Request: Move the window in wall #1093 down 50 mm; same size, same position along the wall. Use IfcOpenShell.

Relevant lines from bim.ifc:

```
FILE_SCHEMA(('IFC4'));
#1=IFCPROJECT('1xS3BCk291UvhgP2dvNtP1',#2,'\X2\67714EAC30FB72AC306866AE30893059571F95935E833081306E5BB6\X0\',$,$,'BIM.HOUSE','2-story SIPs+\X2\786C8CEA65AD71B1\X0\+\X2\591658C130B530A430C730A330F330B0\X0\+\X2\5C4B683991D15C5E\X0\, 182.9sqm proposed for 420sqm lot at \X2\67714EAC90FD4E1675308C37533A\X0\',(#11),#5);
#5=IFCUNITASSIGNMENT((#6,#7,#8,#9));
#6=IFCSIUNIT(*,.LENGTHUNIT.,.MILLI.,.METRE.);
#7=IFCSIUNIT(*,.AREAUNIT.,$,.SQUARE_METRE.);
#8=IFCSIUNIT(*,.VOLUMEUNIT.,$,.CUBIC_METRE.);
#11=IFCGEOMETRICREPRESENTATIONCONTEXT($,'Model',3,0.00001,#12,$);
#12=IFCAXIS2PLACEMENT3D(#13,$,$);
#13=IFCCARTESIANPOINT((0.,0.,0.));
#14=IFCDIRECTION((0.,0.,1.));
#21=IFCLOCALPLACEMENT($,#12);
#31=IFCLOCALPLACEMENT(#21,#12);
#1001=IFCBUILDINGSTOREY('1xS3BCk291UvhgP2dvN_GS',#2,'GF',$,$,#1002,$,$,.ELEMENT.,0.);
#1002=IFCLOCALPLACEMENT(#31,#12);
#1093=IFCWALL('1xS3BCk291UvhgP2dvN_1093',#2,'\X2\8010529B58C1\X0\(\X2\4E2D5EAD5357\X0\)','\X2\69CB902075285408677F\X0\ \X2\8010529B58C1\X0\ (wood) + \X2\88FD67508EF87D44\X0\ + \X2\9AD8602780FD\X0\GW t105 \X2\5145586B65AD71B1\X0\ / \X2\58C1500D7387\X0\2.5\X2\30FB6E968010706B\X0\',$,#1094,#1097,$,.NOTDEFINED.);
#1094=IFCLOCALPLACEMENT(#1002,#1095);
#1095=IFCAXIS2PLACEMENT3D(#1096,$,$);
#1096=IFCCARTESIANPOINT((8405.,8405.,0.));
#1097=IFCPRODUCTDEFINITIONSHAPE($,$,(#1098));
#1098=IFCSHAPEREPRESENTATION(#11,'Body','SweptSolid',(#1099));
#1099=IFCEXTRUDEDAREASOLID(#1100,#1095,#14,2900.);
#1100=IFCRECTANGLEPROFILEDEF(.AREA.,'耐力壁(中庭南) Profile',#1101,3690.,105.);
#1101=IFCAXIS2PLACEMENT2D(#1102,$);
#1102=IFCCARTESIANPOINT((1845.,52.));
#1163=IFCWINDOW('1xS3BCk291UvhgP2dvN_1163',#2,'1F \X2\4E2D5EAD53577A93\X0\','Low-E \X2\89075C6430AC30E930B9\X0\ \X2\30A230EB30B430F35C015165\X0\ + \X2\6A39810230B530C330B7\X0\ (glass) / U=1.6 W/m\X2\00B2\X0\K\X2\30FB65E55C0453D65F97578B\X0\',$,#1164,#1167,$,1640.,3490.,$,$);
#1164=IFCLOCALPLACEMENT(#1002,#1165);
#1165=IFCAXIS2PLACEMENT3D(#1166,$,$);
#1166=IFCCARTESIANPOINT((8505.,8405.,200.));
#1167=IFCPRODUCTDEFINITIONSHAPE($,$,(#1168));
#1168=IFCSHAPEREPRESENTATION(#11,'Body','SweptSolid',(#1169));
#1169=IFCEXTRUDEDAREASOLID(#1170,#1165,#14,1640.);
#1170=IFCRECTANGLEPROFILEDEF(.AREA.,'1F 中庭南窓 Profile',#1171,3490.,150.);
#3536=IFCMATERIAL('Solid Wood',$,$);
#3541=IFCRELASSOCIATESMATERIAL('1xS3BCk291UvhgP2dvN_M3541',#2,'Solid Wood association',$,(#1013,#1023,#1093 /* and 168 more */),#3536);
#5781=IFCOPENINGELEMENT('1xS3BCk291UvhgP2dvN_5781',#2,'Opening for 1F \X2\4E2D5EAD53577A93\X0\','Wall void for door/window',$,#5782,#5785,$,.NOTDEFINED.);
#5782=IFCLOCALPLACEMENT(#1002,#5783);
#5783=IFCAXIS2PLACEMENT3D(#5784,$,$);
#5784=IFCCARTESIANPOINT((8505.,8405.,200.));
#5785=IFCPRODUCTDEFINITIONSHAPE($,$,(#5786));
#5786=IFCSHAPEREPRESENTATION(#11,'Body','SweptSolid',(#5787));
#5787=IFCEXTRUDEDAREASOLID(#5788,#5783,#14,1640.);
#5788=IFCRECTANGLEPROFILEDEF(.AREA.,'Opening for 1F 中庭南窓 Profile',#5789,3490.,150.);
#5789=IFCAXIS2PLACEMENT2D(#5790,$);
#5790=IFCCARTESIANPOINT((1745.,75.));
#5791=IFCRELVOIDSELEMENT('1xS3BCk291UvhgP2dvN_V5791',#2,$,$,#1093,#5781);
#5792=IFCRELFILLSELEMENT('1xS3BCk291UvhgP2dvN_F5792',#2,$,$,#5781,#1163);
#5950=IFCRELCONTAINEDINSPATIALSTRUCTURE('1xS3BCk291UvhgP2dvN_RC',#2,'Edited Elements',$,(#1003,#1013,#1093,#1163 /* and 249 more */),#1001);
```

```python
import numpy as np
import ifcopenshell
import ifcopenshell.api.geometry
import ifcopenshell.util.placement
import ifcopenshell.util.unit

model = ifcopenshell.open("bim.ifc")
unit_scale = ifcopenshell.util.unit.calculate_unit_scale(model)

window = model.by_id(1163)
opening = window.FillsVoids[0].RelatingOpeningElement
dz = -50.0

shift = np.array([0.0, 0.0, dz])
# The window is not placed relative to its opening, so move both.
for product in (opening, window):
    matrix = ifcopenshell.util.placement.get_local_placement(product.ObjectPlacement)
    matrix[:3, 3] += shift
    ifcopenshell.api.geometry.edit_object_placement(model, product=product, matrix=matrix, is_si=False)

print(f"moved by {dz * unit_scale:+.3f} m")

model.write("bim_updated.ifc")
```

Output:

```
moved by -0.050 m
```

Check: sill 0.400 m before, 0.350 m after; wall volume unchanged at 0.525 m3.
